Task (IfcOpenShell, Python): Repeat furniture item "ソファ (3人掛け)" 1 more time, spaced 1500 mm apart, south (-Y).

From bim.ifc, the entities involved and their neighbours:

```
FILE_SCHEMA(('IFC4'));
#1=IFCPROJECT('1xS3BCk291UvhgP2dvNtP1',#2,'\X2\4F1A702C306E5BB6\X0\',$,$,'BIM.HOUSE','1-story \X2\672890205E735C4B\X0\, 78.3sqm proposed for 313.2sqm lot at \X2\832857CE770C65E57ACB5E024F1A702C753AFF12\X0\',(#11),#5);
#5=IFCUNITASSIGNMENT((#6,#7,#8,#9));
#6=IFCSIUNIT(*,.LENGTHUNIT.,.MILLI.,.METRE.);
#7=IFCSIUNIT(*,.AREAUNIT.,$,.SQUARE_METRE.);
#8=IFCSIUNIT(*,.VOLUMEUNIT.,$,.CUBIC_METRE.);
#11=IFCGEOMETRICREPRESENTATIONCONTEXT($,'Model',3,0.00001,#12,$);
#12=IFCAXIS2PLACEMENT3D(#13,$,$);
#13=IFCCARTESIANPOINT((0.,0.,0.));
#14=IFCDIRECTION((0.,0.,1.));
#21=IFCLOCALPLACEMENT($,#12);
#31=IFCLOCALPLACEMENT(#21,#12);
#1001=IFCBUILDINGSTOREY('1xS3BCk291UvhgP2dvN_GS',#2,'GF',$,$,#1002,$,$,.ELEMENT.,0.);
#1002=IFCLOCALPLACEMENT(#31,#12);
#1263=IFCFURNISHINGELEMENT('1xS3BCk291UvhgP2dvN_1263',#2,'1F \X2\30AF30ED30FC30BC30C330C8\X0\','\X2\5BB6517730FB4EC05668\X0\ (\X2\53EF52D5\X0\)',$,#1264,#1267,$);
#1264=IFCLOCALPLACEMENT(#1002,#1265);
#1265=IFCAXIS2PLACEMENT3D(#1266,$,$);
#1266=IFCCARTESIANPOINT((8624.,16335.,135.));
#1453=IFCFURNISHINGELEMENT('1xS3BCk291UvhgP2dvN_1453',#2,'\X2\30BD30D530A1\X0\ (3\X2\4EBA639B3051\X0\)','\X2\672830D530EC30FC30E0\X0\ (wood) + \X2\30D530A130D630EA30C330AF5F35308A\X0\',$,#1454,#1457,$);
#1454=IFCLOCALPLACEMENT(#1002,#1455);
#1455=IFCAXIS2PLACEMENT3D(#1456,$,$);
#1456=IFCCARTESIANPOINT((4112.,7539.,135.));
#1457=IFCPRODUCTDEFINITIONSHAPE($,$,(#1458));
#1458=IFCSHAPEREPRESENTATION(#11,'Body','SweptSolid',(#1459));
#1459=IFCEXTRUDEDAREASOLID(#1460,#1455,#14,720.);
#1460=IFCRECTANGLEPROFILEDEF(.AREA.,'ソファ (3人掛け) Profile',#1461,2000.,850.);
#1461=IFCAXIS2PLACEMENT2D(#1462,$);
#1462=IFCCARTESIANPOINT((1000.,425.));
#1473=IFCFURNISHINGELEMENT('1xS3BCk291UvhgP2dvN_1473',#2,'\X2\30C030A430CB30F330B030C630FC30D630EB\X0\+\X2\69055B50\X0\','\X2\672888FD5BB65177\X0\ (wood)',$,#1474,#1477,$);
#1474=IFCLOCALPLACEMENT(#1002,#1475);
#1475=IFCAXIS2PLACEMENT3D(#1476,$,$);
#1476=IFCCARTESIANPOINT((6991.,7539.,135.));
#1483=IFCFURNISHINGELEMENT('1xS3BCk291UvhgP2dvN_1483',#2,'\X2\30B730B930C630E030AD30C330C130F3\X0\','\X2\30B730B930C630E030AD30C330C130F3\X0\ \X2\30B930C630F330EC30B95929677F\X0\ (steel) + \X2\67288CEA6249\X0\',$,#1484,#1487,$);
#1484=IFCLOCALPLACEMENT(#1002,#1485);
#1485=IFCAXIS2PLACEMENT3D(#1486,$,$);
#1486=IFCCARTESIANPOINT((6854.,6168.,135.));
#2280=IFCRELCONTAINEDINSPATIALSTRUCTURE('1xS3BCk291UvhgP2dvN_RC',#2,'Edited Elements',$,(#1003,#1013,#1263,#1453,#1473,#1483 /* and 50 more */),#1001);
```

```python
import numpy as np
import ifcopenshell
import ifcopenshell.api.geometry
import ifcopenshell.api.root
import ifcopenshell.util.element
import ifcopenshell.util.placement
import ifcopenshell.util.unit

model = ifcopenshell.open("bim.ifc")
unit_scale = ifcopenshell.util.unit.calculate_unit_scale(model)


def reuse_history(source, copy):
    """copy_class also copies each property set's owner history, people and application; keep the originals."""
    for rel in copy.IsDefinedBy:
        if rel.is_a("IfcRelDefinesByProperties") and (history := rel.RelatingPropertyDefinition.OwnerHistory):
            rel.RelatingPropertyDefinition.OwnerHistory = source.OwnerHistory
            ifcopenshell.util.element.remove_deep2(model, history)


source = model.by_id(1453)
base = ifcopenshell.util.placement.get_local_placement(source.ObjectPlacement)
step = np.array([0.0, -1.0, 0.0]) * 1.5 / unit_scale

for i in range(1, 2):
    copy = ifcopenshell.api.root.copy_class(model, product=source)
    copy.Representation = ifcopenshell.util.element.copy_deep(
        model, source.Representation, exclude=["IfcGeometricRepresentationContext", "IfcRepresentationMap"]
    )
    reuse_history(source, copy)
    matrix = base.copy()
    matrix[:3, 3] += i * step
    print("added at", matrix[:3, 3].round(3) + 0.0)
    ifcopenshell.api.geometry.edit_object_placement(model, product=copy, matrix=matrix, is_si=False)

model.write("bim_v2.ifc")
```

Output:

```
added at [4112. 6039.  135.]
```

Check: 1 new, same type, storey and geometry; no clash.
